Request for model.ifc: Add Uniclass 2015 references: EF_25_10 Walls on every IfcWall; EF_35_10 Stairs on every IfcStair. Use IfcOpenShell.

First a look at what the model holds.

```python
import ifcopenshell

model = ifcopenshell.open("model.ifc")
print(model.schema)
print("classifications:", [c.Name for c in model.by_type("IfcClassification")])
for ifc_class in ("IfcDoor", "IfcRoof", "IfcStair", "IfcWall", "IfcWindow"):
    print(ifc_class, len(model.by_type(ifc_class)))
```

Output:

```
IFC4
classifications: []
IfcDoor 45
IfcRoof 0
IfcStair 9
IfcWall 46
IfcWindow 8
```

```python
import ifcopenshell
import ifcopenshell.api.classification

model = ifcopenshell.open("model.ifc")

system = ifcopenshell.api.classification.add_classification(model, classification="Uniclass 2015")

codes = {
    "IfcWall": ("EF_25_10", "Walls"),
    "IfcStair": ("EF_35_10", "Stairs"),
}
for ifc_class, (code, name) in codes.items():
    products = model.by_type(ifc_class)
    ifcopenshell.api.classification.add_reference(
        model, products=products, classification=system, identification=code, name=name
    )
    print(code, len(products))

model.write("model_rev.ifc")
```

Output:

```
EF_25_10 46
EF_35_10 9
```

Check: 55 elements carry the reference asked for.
